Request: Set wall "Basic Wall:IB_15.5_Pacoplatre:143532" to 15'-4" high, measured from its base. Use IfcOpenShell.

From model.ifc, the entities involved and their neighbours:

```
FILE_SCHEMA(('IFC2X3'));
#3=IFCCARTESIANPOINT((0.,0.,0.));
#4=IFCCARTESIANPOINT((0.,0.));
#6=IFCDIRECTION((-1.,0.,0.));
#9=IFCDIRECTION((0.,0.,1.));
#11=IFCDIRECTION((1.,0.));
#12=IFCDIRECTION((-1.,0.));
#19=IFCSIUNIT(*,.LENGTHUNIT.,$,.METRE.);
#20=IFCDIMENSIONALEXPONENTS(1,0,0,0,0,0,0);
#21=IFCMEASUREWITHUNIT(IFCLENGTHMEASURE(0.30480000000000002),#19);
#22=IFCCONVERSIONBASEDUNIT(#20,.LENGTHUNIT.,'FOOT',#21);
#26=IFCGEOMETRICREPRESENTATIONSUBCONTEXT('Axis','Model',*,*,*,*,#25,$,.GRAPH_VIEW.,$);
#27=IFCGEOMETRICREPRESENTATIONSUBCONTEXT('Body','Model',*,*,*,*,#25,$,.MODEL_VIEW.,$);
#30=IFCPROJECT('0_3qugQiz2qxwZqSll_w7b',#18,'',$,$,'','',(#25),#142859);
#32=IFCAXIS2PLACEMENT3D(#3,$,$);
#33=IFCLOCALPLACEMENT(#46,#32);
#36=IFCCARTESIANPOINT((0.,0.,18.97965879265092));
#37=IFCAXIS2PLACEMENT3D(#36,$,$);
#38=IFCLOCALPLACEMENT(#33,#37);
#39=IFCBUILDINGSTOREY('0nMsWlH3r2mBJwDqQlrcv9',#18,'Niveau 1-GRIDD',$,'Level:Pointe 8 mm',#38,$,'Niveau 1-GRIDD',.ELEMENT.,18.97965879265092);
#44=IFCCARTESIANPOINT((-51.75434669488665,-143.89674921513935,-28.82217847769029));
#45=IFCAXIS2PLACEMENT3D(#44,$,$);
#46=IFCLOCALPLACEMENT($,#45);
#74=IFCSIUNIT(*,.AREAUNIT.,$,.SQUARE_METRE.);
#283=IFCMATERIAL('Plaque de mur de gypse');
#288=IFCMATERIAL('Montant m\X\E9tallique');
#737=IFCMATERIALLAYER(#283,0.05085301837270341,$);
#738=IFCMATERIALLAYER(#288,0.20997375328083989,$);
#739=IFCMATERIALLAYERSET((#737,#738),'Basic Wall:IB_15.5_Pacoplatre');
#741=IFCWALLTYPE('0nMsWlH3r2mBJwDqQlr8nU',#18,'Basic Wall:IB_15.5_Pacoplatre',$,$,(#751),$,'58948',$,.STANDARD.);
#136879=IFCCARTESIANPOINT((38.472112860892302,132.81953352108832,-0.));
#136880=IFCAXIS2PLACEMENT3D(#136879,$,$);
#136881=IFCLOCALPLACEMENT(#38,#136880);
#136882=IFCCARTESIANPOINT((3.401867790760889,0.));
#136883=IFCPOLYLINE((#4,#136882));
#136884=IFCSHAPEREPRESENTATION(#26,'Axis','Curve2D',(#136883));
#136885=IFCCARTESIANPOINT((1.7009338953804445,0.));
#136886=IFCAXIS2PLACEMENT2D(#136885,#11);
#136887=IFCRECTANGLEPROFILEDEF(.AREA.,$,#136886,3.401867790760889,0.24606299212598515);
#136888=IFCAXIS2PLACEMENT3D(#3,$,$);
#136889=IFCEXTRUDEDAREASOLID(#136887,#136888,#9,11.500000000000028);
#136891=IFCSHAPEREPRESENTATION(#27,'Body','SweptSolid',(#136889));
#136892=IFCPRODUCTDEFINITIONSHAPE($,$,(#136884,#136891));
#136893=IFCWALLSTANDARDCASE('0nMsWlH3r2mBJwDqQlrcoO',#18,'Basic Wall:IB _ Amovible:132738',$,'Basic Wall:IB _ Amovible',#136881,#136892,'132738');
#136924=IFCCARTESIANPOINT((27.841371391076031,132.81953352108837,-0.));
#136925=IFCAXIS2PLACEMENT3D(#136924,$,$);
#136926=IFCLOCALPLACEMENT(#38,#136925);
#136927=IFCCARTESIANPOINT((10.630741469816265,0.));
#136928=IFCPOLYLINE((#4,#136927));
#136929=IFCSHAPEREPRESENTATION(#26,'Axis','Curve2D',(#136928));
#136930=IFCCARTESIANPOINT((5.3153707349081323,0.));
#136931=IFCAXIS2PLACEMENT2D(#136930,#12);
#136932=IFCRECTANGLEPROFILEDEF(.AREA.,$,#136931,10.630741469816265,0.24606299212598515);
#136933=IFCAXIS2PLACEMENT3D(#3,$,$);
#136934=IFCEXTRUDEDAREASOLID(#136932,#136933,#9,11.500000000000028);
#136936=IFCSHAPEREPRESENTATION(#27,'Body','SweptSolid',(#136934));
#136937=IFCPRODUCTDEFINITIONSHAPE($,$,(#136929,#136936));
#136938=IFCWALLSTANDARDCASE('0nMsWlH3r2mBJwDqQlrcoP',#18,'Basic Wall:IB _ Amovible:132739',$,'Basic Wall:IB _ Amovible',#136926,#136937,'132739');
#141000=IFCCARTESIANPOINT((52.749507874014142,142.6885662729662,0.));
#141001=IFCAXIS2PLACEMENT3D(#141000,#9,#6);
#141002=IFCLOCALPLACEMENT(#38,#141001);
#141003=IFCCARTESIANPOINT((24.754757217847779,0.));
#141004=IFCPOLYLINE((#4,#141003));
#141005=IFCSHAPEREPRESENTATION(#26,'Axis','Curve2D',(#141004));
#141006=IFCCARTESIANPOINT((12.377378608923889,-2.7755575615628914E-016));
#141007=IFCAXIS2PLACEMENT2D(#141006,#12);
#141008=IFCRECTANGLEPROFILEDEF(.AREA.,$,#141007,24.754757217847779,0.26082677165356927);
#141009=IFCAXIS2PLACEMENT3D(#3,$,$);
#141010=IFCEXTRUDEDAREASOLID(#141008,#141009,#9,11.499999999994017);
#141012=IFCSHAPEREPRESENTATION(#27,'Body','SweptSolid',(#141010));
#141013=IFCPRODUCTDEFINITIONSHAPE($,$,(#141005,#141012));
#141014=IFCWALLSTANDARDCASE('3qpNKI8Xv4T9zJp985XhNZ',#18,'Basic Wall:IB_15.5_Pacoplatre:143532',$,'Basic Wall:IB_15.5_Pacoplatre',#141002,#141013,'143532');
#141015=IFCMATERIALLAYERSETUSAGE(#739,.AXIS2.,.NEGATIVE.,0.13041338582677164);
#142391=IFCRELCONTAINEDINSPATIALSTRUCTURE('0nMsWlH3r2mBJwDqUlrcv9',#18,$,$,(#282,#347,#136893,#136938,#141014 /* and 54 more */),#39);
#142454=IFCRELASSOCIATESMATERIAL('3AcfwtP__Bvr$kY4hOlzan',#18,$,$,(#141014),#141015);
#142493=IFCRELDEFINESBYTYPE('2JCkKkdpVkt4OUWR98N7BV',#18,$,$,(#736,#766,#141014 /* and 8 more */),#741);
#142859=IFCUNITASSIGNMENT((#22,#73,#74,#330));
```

```python
import ifcopenshell
import ifcopenshell.geom
import ifcopenshell.util.representation
import ifcopenshell.util.shape
import ifcopenshell.util.unit

model = ifcopenshell.open("model.ifc")
unit_scale = ifcopenshell.util.unit.calculate_unit_scale(model)
settings = ifcopenshell.geom.settings()


def volume(element):
    """Net volume in cubic metres, openings subtracted."""
    shape = ifcopenshell.geom.create_shape(settings, element)
    return ifcopenshell.util.shape.get_volume(shape.geometry)


wall = model.by_guid("3qpNKI8Xv4T9zJp985XhNZ")
before = volume(wall)

body = ifcopenshell.util.representation.get_representation(wall, "Model", "Body")
solid = body.Items[0]
old_height = solid.Depth
solid.Depth = 184 * 0.0254 / unit_scale
after = volume(wall)

print(f"height {old_height:g} -> {solid.Depth:g}, volume {before:.3f} -> {after:.3f} m3")

model.write("model_updated.ifc")
```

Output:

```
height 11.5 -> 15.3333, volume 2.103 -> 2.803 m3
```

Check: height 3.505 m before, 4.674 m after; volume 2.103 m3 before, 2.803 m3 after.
